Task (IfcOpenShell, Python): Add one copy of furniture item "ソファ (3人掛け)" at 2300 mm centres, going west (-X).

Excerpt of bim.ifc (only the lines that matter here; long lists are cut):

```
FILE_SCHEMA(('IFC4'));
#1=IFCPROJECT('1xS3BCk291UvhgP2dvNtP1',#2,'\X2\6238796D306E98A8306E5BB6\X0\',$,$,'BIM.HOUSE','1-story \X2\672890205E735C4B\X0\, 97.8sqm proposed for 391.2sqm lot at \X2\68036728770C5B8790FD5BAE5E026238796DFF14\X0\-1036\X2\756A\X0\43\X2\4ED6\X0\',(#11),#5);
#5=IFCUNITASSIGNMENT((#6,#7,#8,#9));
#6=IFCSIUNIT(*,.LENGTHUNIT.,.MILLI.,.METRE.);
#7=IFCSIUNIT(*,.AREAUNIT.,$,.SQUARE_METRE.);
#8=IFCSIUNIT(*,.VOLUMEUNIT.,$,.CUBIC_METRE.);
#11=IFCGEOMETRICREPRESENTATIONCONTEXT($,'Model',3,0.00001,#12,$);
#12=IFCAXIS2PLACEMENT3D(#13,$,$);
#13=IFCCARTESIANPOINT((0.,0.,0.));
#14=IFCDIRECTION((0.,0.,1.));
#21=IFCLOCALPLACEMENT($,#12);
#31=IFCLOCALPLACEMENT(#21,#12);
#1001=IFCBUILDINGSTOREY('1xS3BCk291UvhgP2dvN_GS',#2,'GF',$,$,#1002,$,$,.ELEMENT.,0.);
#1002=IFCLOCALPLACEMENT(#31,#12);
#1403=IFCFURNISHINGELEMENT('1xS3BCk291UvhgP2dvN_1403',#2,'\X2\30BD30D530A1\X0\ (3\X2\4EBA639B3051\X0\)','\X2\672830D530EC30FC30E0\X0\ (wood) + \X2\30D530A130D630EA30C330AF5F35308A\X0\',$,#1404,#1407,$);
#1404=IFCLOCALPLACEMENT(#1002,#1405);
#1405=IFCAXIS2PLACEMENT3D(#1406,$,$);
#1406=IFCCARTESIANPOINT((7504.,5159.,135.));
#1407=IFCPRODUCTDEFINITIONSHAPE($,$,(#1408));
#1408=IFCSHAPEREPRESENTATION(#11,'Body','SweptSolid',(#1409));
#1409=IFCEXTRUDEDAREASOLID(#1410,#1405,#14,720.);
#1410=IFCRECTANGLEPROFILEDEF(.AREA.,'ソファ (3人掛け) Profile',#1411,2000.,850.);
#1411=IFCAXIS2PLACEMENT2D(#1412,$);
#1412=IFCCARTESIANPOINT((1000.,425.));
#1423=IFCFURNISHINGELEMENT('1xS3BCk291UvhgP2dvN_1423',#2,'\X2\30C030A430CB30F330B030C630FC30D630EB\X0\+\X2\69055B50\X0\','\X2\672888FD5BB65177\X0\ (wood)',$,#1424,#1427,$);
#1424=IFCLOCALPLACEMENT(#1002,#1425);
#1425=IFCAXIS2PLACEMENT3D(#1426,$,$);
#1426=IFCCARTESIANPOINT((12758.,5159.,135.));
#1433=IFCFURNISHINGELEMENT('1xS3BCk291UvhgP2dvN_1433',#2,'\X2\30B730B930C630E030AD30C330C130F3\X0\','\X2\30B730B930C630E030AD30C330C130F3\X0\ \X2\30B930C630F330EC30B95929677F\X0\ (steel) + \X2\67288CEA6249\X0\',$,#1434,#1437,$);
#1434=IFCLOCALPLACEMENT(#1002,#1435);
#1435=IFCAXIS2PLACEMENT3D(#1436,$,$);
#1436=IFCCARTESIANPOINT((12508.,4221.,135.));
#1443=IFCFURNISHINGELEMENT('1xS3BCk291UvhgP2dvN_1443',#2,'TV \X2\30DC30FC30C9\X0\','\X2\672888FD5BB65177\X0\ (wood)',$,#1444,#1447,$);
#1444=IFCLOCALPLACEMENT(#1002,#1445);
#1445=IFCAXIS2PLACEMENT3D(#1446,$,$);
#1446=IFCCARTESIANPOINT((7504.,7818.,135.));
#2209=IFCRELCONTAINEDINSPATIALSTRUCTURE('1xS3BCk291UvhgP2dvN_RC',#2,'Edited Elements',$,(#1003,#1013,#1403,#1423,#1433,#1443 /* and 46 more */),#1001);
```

```python
import numpy as np
import ifcopenshell
import ifcopenshell.api.geometry
import ifcopenshell.api.root
import ifcopenshell.util.element
import ifcopenshell.util.placement

model = ifcopenshell.open("bim.ifc")


def reuse_history(source, copy):
    """copy_class also copies each property set's owner history, people and application; keep the originals."""
    for rel in copy.IsDefinedBy:
        if rel.is_a("IfcRelDefinesByProperties") and (history := rel.RelatingPropertyDefinition.OwnerHistory):
            rel.RelatingPropertyDefinition.OwnerHistory = source.OwnerHistory
            ifcopenshell.util.element.remove_deep2(model, history)


source = model.by_id(1403)
base = ifcopenshell.util.placement.get_local_placement(source.ObjectPlacement)
step = np.array([-1.0, 0.0, 0.0]) * 2300.0

for i in range(1, 2):
    copy = ifcopenshell.api.root.copy_class(model, product=source)
    copy.Representation = ifcopenshell.util.element.copy_deep(
        model, source.Representation, exclude=["IfcGeometricRepresentationContext", "IfcRepresentationMap"]
    )
    reuse_history(source, copy)
    matrix = base.copy()
    matrix[:3, 3] += i * step
    print("added at", matrix[:3, 3].round(3) + 0.0)
    ifcopenshell.api.geometry.edit_object_placement(model, product=copy, matrix=matrix, is_si=False)

model.write("bim_v2.ifc")
```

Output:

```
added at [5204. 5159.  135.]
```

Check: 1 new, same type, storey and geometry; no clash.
